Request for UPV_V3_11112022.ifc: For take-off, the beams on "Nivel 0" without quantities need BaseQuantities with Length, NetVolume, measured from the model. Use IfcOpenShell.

First a look at what the model holds.

```python
import ifcopenshell
import ifcopenshell.util.element
import ifcopenshell.util.unit

model = ifcopenshell.open("UPV_V3_11112022.ifc")
print(model.schema)
for unit_type in ("LENGTHUNIT", "AREAUNIT", "VOLUMEUNIT"):
    print(unit_type, ifcopenshell.util.unit.calculate_unit_scale(model, unit_type))
storey = next(s for s in model.by_type("IfcBuildingStorey") if s.Name == "Nivel 0")
beams = [e for e in ifcopenshell.util.element.get_decomposition(storey) if e.is_a("IfcBeam")]
for e in sorted(beams, key=lambda e: e.id()):
    print(e.id(), e.is_a(), e.Name, list(ifcopenshell.util.element.get_psets(e, qtos_only=True)), sep=" | ")
```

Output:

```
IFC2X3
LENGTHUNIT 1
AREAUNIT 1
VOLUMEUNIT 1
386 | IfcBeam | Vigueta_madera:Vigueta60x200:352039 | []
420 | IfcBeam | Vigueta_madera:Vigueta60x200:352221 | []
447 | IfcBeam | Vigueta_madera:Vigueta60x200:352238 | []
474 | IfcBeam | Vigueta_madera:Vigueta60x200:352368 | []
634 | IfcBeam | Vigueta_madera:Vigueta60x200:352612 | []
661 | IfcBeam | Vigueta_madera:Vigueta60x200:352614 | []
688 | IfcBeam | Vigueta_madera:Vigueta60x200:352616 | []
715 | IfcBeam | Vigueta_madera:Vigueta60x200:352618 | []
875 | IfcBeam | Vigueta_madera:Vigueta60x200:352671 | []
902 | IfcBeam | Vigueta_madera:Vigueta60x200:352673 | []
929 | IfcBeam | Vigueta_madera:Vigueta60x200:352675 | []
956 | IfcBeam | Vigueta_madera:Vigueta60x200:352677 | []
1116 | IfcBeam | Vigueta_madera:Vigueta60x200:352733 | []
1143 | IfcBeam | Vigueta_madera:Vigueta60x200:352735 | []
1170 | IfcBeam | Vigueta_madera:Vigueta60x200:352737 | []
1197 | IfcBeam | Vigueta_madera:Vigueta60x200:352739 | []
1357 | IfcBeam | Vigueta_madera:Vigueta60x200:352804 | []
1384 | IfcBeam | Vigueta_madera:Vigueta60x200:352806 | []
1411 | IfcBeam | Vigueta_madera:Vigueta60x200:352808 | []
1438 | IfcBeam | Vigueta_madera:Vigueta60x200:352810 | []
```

```python
import ifcopenshell
import ifcopenshell.api.pset
import ifcopenshell.geom
import ifcopenshell.util.element
import ifcopenshell.util.shape
import ifcopenshell.util.unit

model = ifcopenshell.open("UPV_V3_11112022.ifc")
unit_scale = ifcopenshell.util.unit.calculate_unit_scale(model)
volume_scale = ifcopenshell.util.unit.calculate_unit_scale(model, "VOLUMEUNIT")
settings = ifcopenshell.geom.settings()

storey = next(s for s in model.by_type("IfcBuildingStorey") if s.Name == "Nivel 0")
beams = [e for e in ifcopenshell.util.element.get_decomposition(storey) if e.is_a("IfcBeam")]

for e in sorted(beams, key=lambda e: e.id()):
    if ifcopenshell.util.element.get_psets(e, qtos_only=True, should_inherit=False):
        continue
    # Geometry comes back in metres, in the element's own axes.
    shape = ifcopenshell.geom.create_shape(settings, e)
    values = {
        "Length": ifcopenshell.util.shape.get_max_xyz(shape.geometry) / unit_scale,
        "NetVolume": ifcopenshell.util.shape.get_volume(shape.geometry) / volume_scale,
    }
    qto = ifcopenshell.api.pset.add_qto(model, product=e, name="BaseQuantities")
    ifcopenshell.api.pset.edit_qto(model, qto=qto, properties=values)
    print(e.id(), {k: round(v, 3) for k, v in values.items()})

model.write("UPV_V3_11112022_rev.ifc")
```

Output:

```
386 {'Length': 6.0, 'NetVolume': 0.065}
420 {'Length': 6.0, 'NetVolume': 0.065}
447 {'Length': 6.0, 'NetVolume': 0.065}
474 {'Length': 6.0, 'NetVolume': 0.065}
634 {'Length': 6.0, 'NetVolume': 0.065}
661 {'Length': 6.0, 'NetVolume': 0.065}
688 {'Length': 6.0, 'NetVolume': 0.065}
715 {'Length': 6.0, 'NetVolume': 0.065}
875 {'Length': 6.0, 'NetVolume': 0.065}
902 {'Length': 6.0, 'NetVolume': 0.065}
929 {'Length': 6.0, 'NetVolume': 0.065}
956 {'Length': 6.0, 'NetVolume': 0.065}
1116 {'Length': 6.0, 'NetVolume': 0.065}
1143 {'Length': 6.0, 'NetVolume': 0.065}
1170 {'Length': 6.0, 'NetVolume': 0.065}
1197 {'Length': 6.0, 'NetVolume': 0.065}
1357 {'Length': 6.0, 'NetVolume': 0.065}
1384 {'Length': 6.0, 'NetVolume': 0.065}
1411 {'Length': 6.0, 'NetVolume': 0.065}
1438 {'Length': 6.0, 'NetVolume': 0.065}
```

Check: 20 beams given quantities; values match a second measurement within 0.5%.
